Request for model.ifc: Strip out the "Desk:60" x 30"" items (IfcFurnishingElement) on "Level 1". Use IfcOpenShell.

First a look at what the model holds.

```python
import ifcopenshell
import ifcopenshell.util.element

model = ifcopenshell.open("model.ifc")
print(model.schema)
storey = next(s for s in model.by_type("IfcBuildingStorey") if s.Name == "Level 1")
furniture = [e for e in ifcopenshell.util.element.get_decomposition(storey) if e.is_a("IfcFurnishingElement")]
seen = {}
for e in furniture:
    element_type = ifcopenshell.util.element.get_type(e)
    name = element_type.Name if element_type not in (None, e) else None
    seen[name] = seen.get(name, 0) + 1
for name, count in sorted(seen.items(), key=str):
    print(count, "x", name)
```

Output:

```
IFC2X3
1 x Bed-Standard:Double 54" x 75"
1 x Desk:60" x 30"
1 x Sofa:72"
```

```python
import ifcopenshell
import ifcopenshell.api.root
import ifcopenshell.util.element

model = ifcopenshell.open("model.ifc")

storey = next(s for s in model.by_type("IfcBuildingStorey") if s.Name == "Level 1")
furniture = [e for e in ifcopenshell.util.element.get_decomposition(storey) if e.is_a("IfcFurnishingElement")]
targets = [e for e in furniture if (t := ifcopenshell.util.element.get_type(e)) not in (None, e) and t.Name == 'Desk:60" x 30"']

for e in targets:
    ifcopenshell.api.root.remove_product(model, product=e)
print(len(targets), "removed")

model.write("model-out.ifc")
```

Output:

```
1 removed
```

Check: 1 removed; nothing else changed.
